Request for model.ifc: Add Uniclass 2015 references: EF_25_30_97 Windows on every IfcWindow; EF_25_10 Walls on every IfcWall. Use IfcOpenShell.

First a look at what the model holds.

```python
import ifcopenshell

model = ifcopenshell.open("model.ifc")
print(model.schema)
print("classifications:", [c.Name for c in model.by_type("IfcClassification")])
for ifc_class in ("IfcDoor", "IfcRoof", "IfcStair", "IfcWall", "IfcWindow"):
    print(ifc_class, len(model.by_type(ifc_class)))
```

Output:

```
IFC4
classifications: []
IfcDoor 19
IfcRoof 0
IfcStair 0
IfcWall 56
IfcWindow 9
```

```python
import ifcopenshell
import ifcopenshell.api.classification

model = ifcopenshell.open("model.ifc")

system = ifcopenshell.api.classification.add_classification(model, classification="Uniclass 2015")

codes = {
    "IfcWindow": ("EF_25_30_97", "Windows"),
    "IfcWall": ("EF_25_10", "Walls"),
}
for ifc_class, (code, name) in codes.items():
    products = model.by_type(ifc_class)
    ifcopenshell.api.classification.add_reference(
        model, products=products, classification=system, identification=code, name=name
    )
    print(code, len(products))

model.write("model_rev.ifc")
```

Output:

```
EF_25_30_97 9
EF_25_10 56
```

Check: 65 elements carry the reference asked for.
